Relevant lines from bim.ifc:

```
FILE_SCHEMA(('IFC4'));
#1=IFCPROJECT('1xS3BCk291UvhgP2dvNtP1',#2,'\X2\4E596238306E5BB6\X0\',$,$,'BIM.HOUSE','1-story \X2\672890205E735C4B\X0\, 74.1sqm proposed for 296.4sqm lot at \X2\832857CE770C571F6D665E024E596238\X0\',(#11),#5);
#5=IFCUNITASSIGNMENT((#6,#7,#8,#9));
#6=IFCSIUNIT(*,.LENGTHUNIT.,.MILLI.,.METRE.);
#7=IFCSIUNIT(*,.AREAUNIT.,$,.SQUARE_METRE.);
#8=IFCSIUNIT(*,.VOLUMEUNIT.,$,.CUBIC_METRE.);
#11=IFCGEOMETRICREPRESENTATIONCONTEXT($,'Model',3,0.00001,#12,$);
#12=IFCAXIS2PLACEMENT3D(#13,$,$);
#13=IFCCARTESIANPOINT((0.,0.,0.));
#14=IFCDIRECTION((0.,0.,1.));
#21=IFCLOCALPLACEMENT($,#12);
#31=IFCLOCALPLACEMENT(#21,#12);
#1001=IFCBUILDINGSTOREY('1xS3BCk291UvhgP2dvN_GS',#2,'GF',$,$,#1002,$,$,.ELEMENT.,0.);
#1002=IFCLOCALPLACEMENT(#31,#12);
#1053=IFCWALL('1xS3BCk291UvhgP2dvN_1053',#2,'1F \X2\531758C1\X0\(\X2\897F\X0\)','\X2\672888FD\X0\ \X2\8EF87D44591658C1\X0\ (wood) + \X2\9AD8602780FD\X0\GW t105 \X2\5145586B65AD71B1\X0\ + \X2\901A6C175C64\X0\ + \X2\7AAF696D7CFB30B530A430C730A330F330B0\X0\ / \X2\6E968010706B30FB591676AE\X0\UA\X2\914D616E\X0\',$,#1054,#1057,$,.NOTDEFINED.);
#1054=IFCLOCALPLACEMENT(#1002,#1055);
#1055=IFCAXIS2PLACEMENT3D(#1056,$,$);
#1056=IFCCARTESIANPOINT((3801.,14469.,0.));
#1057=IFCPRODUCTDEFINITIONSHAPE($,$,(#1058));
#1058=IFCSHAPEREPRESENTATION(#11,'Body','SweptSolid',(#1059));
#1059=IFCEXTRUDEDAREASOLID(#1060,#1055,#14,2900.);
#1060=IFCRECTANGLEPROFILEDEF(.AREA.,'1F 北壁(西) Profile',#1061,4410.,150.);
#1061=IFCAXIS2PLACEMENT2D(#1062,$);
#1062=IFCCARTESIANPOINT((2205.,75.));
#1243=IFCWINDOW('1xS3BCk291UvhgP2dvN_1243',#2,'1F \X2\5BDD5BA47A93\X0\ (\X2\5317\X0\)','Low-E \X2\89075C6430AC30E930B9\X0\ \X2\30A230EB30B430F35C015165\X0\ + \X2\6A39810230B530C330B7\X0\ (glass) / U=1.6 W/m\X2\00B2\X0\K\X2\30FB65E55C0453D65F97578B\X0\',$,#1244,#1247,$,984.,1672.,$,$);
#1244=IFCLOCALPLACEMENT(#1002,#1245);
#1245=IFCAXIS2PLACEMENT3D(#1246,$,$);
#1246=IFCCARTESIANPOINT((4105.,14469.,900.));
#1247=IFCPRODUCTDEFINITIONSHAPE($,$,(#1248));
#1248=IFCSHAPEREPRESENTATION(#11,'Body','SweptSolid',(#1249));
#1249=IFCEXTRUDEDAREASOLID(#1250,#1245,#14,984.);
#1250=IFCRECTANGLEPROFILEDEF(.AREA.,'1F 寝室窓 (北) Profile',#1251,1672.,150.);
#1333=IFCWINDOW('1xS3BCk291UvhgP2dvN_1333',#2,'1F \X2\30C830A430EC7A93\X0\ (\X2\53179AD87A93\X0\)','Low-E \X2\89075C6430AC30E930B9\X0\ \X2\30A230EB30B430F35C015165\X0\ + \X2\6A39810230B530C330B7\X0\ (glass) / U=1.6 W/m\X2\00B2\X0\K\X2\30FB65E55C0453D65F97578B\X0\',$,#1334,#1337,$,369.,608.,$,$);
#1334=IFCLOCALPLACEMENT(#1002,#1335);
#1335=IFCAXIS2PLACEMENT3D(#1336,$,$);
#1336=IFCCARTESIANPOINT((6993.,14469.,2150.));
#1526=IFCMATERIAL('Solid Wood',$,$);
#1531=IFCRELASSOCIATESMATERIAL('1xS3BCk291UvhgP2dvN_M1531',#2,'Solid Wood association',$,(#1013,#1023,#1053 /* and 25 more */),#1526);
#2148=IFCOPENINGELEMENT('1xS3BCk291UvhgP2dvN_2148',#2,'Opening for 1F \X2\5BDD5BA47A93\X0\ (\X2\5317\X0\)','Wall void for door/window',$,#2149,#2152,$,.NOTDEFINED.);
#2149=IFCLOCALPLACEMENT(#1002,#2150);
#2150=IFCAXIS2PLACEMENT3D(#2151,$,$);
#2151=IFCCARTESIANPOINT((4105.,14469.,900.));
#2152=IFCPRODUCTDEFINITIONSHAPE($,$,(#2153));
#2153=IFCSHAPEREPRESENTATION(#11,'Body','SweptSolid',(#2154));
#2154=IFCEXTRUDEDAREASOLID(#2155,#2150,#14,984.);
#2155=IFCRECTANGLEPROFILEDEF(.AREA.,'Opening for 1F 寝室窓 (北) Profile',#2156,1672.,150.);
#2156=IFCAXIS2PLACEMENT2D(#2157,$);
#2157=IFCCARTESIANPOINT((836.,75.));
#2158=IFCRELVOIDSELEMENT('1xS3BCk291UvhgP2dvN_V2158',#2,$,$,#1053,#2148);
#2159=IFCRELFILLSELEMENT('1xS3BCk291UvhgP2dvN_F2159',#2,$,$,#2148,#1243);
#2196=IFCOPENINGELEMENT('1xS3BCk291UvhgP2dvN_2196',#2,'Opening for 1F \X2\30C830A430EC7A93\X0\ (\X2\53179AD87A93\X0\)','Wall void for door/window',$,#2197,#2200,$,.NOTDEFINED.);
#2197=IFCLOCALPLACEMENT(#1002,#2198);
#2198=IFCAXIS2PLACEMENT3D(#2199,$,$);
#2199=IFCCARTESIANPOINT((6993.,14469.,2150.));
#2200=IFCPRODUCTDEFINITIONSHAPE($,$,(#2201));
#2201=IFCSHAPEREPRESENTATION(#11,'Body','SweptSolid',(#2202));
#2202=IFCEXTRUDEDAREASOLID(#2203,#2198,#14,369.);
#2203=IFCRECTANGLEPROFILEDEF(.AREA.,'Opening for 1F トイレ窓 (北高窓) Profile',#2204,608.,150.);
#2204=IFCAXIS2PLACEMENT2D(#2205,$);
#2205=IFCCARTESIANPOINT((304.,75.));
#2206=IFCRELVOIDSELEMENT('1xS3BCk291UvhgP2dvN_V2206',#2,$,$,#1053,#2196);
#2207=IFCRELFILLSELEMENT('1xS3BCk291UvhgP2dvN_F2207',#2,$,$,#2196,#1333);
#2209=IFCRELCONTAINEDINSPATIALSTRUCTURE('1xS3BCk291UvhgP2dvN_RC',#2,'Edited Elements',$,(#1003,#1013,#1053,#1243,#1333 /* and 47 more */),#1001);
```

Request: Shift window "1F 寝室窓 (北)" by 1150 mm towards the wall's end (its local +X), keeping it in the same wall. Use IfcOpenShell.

```python
import ifcopenshell
import ifcopenshell.api.geometry
import ifcopenshell.util.placement

model = ifcopenshell.open("bim.ifc")

window = model.by_guid("1xS3BCk291UvhgP2dvN_1243")
opening = window.FillsVoids[0].RelatingOpeningElement
wall = opening.VoidsElements[0].RelatingBuildingElement

wall_matrix = ifcopenshell.util.placement.get_local_placement(wall.ObjectPlacement)
shift = wall_matrix[:3, 0] * 1150.0
before = ifcopenshell.util.placement.get_local_placement(window.ObjectPlacement)[:3, 3].copy()

# The window is not placed relative to its opening, so move both.
for product in (opening, window):
    matrix = ifcopenshell.util.placement.get_local_placement(product.ObjectPlacement)
    matrix[:3, 3] += shift
    ifcopenshell.api.geometry.edit_object_placement(model, product=product, matrix=matrix, is_si=False)

after = ifcopenshell.util.placement.get_local_placement(window.ObjectPlacement)[:3, 3]
print("window moved by", (after - before).round(3) + 0.0)

model.write("bim-out.ifc")
```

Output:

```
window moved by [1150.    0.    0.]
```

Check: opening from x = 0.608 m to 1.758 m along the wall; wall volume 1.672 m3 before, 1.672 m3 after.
